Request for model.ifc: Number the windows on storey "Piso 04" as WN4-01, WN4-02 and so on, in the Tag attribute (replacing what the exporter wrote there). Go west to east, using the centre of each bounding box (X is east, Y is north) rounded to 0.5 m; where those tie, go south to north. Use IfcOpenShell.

First a look at what the model holds.

```python
import ifcopenshell
import ifcopenshell.util.element
import ifcopenshell.util.placement

model = ifcopenshell.open("model.ifc")
print(model.schema)
storey = next(s for s in model.by_type("IfcBuildingStorey") if s.Name == "Piso 04")
windows = [e for e in ifcopenshell.util.element.get_decomposition(storey) if e.is_a("IfcWindow")]
for e in sorted(windows, key=lambda e: e.id()):
    origin = ifcopenshell.util.placement.get_local_placement(e.ObjectPlacement)[:3, 3]
    print(e.id(), e.Tag, e.Name, origin.round(2) + 0.0, sep=" | ")
```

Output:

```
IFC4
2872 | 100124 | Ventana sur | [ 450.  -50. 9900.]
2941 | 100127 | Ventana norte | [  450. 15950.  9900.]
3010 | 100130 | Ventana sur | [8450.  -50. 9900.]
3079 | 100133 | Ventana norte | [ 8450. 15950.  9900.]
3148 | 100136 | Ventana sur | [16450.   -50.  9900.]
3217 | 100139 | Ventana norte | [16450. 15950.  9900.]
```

```python
import ifcopenshell
import ifcopenshell.geom
import ifcopenshell.util.element
import ifcopenshell.util.shape

model = ifcopenshell.open("model.ifc")
settings = ifcopenshell.geom.settings()
settings.set("use-world-coords", True)


def centre(element):
    shape = ifcopenshell.geom.create_shape(settings, element)
    return ifcopenshell.util.shape.get_bbox_centroid(shape.geometry)


storey = next(s for s in model.by_type("IfcBuildingStorey") if s.Name == "Piso 04")
windows = [e for e in ifcopenshell.util.element.get_decomposition(storey) if e.is_a("IfcWindow")]

# Insertion points can sit at a corner or the storey origin, so sort by the geometry (in metres).
centres = {e: centre(e) for e in windows}
windows.sort(key=lambda e: (round(centres[e][0] / 0.5), centres[e][1]))

for i, e in enumerate(windows, start=1):
    number = f"WN4-{i:02d}"
    e.Tag = number
    print(e.id(), number)

model.write("model_edited.ifc")
```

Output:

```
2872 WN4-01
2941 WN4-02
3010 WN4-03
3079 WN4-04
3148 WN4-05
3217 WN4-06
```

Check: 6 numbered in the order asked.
